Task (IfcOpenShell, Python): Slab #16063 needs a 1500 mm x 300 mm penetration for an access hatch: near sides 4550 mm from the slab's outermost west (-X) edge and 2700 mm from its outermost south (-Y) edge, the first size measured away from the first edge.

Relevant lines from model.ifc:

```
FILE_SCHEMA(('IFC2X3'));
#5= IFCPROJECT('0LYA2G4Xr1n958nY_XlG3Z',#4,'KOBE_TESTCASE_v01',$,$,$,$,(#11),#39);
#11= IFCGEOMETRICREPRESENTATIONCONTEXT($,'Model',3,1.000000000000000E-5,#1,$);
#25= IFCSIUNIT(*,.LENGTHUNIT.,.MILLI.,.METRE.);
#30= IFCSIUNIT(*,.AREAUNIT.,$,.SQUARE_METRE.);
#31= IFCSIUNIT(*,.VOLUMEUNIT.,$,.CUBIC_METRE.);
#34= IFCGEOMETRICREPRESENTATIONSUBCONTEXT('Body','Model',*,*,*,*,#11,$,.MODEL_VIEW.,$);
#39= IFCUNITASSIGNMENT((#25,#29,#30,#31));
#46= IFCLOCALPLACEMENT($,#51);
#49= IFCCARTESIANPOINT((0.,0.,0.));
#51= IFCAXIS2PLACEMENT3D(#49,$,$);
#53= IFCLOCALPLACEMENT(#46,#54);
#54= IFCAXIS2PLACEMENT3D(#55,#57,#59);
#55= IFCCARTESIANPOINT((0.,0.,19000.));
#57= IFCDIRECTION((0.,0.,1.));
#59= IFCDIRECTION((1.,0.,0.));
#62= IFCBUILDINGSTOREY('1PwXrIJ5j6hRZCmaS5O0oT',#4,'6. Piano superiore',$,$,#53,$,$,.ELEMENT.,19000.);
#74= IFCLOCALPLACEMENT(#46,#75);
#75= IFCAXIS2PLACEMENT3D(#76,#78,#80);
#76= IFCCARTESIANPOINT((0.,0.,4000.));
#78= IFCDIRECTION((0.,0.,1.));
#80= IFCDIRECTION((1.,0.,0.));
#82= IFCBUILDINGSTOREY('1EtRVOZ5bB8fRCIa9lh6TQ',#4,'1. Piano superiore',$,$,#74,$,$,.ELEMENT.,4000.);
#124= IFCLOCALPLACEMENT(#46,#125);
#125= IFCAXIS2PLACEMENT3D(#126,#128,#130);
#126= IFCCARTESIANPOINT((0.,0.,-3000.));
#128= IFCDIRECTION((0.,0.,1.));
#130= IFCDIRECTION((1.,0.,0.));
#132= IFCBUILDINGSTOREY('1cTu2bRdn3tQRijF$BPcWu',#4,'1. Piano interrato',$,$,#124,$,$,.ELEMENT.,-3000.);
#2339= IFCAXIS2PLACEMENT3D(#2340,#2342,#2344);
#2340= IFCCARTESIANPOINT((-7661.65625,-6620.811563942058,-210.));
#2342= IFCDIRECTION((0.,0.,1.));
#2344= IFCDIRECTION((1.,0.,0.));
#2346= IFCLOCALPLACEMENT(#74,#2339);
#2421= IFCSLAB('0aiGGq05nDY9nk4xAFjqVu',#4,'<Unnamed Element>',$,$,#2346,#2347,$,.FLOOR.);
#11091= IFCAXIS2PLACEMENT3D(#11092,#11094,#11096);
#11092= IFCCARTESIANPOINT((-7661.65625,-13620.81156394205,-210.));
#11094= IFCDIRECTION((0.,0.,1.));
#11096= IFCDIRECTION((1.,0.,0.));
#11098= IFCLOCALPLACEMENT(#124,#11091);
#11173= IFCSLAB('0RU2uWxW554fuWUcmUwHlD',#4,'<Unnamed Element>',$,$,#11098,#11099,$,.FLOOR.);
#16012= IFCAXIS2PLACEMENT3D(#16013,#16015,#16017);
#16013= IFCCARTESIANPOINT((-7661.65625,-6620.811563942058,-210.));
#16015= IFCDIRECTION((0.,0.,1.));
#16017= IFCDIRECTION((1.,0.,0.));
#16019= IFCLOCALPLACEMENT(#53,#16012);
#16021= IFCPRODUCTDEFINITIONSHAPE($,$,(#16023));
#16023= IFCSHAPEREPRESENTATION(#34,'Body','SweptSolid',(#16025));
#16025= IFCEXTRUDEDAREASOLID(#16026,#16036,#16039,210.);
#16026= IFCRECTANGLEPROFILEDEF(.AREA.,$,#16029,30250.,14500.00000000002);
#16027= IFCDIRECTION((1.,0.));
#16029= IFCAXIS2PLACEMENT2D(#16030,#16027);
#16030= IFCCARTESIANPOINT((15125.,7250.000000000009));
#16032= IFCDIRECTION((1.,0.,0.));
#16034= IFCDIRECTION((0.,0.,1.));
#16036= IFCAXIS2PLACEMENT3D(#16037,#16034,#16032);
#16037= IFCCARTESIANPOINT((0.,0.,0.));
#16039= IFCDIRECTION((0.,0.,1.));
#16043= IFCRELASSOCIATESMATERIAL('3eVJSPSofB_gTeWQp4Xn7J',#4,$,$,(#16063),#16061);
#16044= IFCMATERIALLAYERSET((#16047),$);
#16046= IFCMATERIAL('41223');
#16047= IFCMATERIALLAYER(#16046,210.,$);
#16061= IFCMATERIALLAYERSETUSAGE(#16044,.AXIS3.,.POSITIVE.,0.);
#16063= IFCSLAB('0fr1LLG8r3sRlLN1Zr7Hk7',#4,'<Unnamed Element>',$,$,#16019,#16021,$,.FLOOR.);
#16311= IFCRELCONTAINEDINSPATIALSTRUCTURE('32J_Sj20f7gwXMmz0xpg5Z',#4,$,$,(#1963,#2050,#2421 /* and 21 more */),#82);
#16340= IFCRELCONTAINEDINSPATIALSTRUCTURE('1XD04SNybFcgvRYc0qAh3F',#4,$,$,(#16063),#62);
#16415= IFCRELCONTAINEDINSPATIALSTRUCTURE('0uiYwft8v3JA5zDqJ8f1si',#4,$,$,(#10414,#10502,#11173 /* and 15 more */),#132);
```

```python
import numpy as np
import ifcopenshell
import ifcopenshell.api.feature
import ifcopenshell.api.geometry
import ifcopenshell.api.root
import ifcopenshell.geom
import ifcopenshell.util.placement
import ifcopenshell.util.representation
import ifcopenshell.util.shape
import ifcopenshell.util.unit

model = ifcopenshell.open("model.ifc")
unit_scale = ifcopenshell.util.unit.calculate_unit_scale(model)
settings = ifcopenshell.geom.settings()


def volume(element):
    """Net volume in cubic metres, openings subtracted."""
    shape = ifcopenshell.geom.create_shape(settings, element)
    return ifcopenshell.util.shape.get_volume(shape.geometry)


slab = model.by_guid("0fr1LLG8r3sRlLN1Zr7Hk7")
before = volume(slab)

# Extent in the slab's own axes, in metres. The edges named are its -X and -Y sides.
slab_shape = ifcopenshell.geom.create_shape(settings, slab)
vertices = ifcopenshell.util.shape.get_vertices(slab_shape.geometry)
x_min, y_min, bottom = vertices.min(axis=0)
top = vertices[:, 2].max()

opening = ifcopenshell.api.root.create_entity(model, ifc_class="IfcOpeningElement", name="Access hatch opening")
context = ifcopenshell.util.representation.get_context(model, "Model", "Body", "MODEL_VIEW")
width, depth = 1.5, 0.3
outline = [(0.0, 0.0), (width, 0.0), (width, depth), (0.0, depth), (0.0, 0.0)]
# Overshoot both faces by 50 mm so the cut is clean.
shape = ifcopenshell.api.geometry.add_slab_representation(
    model, context=context, depth=top - bottom + 0.1, polyline=outline
)
ifcopenshell.api.geometry.assign_representation(model, product=opening, representation=shape)

matrix = ifcopenshell.util.placement.get_local_placement(slab.ObjectPlacement)
matrix[:, 3] = matrix @ np.append(np.array([x_min + 4.55, y_min + 2.7, bottom - 0.05]) / unit_scale, 1.0)
ifcopenshell.api.geometry.edit_object_placement(model, product=opening, matrix=matrix, is_si=False)
ifcopenshell.api.feature.add_feature(model, feature=opening, element=slab)

after = volume(slab)

print(f"slab volume {before:.3f} -> {after:.3f} m3")

model.write("model_edited.ifc")
```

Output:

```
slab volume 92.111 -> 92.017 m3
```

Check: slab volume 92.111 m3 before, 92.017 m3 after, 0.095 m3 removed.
